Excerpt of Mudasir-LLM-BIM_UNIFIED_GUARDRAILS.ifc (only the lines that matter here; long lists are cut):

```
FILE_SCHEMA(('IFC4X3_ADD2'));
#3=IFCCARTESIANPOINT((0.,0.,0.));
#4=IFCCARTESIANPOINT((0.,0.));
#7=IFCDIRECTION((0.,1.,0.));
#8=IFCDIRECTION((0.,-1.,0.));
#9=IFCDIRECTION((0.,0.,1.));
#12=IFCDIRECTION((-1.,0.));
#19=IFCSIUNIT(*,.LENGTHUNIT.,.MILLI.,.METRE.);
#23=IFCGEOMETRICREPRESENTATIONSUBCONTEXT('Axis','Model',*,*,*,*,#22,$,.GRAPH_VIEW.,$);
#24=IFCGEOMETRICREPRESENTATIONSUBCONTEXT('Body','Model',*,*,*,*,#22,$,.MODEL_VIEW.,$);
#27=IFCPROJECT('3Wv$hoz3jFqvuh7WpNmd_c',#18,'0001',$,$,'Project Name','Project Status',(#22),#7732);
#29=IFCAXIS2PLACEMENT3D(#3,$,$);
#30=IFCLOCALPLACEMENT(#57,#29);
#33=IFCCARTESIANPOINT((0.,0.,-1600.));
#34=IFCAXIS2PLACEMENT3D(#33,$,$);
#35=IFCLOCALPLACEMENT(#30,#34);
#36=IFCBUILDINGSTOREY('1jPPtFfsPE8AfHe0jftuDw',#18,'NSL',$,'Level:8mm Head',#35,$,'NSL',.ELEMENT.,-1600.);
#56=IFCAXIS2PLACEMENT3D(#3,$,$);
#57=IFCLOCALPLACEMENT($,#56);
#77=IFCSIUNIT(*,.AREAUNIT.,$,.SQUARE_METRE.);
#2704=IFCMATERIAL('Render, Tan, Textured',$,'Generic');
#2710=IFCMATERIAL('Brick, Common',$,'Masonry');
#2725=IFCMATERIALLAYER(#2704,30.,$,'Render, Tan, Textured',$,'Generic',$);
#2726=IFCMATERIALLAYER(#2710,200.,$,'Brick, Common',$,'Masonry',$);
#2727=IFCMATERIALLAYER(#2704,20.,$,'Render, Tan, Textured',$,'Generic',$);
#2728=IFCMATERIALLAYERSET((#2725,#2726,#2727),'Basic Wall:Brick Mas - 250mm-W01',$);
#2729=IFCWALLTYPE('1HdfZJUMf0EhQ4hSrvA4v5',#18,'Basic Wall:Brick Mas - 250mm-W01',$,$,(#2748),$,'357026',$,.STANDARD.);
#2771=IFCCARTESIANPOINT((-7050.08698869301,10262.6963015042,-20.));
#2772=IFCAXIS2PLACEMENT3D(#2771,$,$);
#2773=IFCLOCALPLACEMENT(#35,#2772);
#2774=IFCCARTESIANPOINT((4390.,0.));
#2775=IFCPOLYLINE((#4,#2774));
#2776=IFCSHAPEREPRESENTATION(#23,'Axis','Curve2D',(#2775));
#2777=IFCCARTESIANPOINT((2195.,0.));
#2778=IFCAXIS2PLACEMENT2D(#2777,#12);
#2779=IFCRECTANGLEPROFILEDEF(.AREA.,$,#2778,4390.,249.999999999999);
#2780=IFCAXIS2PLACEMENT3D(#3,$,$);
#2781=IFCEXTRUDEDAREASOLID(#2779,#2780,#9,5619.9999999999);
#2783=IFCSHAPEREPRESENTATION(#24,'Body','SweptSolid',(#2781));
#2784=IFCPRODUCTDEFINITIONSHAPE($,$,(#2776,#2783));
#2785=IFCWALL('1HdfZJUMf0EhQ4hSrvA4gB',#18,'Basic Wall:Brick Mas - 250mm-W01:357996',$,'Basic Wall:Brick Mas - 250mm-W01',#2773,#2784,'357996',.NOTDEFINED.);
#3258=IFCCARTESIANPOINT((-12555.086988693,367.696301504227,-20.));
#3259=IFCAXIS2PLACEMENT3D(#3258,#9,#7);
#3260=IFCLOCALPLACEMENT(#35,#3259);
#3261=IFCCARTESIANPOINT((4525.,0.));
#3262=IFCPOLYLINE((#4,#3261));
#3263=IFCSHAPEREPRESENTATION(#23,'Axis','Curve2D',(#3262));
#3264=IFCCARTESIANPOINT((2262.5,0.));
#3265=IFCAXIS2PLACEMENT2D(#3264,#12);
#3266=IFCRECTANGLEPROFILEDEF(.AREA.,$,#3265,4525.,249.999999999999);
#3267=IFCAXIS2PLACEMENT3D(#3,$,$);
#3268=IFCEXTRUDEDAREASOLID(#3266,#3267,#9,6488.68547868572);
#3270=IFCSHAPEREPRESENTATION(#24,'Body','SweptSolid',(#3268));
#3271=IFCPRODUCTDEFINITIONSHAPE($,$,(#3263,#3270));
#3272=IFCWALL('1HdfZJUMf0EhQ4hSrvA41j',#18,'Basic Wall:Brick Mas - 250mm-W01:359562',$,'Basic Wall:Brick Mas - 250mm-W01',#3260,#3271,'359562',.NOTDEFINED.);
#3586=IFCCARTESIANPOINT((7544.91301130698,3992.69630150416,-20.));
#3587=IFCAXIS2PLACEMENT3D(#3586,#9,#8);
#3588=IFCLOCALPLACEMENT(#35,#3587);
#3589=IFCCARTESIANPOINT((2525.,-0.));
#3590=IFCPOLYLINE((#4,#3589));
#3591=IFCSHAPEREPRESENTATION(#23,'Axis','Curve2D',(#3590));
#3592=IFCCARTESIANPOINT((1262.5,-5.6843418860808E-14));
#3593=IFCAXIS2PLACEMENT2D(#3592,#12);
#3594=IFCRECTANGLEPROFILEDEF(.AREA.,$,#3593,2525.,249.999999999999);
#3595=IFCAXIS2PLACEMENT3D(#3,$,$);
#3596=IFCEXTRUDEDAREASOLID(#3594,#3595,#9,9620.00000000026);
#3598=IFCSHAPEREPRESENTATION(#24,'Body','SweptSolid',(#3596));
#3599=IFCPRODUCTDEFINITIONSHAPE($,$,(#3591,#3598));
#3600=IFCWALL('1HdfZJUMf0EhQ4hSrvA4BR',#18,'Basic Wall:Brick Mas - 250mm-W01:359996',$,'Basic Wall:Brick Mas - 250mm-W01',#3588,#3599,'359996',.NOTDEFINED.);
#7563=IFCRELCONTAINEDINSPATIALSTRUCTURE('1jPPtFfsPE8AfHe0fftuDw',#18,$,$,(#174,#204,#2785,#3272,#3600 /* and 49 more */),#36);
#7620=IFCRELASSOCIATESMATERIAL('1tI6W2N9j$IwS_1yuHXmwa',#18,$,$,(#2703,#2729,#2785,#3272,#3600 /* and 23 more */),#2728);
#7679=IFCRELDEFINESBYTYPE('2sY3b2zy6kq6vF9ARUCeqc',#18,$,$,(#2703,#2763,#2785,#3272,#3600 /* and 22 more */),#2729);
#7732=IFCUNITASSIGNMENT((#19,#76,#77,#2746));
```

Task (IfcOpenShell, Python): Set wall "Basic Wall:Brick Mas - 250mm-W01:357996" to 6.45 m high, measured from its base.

```python
import ifcopenshell
import ifcopenshell.geom
import ifcopenshell.util.representation
import ifcopenshell.util.shape
import ifcopenshell.util.unit

model = ifcopenshell.open("Mudasir-LLM-BIM_UNIFIED_GUARDRAILS.ifc")
unit_scale = ifcopenshell.util.unit.calculate_unit_scale(model)
settings = ifcopenshell.geom.settings()


def volume(element):
    """Net volume in cubic metres, openings subtracted."""
    shape = ifcopenshell.geom.create_shape(settings, element)
    return ifcopenshell.util.shape.get_volume(shape.geometry)


wall = model.by_guid("1HdfZJUMf0EhQ4hSrvA4gB")
before = volume(wall)

body = ifcopenshell.util.representation.get_representation(wall, "Model", "Body")
solid = body.Items[0]
old_height = solid.Depth
solid.Depth = 6.45 / unit_scale
after = volume(wall)

print(f"height {old_height:g} -> {solid.Depth:g}, volume {before:.3f} -> {after:.3f} m3")

model.write("Mudasir-LLM-BIM_UNIFIED_GUARDRAILS-out.ifc")
```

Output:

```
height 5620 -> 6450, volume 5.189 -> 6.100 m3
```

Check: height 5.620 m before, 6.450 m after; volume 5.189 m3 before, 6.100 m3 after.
